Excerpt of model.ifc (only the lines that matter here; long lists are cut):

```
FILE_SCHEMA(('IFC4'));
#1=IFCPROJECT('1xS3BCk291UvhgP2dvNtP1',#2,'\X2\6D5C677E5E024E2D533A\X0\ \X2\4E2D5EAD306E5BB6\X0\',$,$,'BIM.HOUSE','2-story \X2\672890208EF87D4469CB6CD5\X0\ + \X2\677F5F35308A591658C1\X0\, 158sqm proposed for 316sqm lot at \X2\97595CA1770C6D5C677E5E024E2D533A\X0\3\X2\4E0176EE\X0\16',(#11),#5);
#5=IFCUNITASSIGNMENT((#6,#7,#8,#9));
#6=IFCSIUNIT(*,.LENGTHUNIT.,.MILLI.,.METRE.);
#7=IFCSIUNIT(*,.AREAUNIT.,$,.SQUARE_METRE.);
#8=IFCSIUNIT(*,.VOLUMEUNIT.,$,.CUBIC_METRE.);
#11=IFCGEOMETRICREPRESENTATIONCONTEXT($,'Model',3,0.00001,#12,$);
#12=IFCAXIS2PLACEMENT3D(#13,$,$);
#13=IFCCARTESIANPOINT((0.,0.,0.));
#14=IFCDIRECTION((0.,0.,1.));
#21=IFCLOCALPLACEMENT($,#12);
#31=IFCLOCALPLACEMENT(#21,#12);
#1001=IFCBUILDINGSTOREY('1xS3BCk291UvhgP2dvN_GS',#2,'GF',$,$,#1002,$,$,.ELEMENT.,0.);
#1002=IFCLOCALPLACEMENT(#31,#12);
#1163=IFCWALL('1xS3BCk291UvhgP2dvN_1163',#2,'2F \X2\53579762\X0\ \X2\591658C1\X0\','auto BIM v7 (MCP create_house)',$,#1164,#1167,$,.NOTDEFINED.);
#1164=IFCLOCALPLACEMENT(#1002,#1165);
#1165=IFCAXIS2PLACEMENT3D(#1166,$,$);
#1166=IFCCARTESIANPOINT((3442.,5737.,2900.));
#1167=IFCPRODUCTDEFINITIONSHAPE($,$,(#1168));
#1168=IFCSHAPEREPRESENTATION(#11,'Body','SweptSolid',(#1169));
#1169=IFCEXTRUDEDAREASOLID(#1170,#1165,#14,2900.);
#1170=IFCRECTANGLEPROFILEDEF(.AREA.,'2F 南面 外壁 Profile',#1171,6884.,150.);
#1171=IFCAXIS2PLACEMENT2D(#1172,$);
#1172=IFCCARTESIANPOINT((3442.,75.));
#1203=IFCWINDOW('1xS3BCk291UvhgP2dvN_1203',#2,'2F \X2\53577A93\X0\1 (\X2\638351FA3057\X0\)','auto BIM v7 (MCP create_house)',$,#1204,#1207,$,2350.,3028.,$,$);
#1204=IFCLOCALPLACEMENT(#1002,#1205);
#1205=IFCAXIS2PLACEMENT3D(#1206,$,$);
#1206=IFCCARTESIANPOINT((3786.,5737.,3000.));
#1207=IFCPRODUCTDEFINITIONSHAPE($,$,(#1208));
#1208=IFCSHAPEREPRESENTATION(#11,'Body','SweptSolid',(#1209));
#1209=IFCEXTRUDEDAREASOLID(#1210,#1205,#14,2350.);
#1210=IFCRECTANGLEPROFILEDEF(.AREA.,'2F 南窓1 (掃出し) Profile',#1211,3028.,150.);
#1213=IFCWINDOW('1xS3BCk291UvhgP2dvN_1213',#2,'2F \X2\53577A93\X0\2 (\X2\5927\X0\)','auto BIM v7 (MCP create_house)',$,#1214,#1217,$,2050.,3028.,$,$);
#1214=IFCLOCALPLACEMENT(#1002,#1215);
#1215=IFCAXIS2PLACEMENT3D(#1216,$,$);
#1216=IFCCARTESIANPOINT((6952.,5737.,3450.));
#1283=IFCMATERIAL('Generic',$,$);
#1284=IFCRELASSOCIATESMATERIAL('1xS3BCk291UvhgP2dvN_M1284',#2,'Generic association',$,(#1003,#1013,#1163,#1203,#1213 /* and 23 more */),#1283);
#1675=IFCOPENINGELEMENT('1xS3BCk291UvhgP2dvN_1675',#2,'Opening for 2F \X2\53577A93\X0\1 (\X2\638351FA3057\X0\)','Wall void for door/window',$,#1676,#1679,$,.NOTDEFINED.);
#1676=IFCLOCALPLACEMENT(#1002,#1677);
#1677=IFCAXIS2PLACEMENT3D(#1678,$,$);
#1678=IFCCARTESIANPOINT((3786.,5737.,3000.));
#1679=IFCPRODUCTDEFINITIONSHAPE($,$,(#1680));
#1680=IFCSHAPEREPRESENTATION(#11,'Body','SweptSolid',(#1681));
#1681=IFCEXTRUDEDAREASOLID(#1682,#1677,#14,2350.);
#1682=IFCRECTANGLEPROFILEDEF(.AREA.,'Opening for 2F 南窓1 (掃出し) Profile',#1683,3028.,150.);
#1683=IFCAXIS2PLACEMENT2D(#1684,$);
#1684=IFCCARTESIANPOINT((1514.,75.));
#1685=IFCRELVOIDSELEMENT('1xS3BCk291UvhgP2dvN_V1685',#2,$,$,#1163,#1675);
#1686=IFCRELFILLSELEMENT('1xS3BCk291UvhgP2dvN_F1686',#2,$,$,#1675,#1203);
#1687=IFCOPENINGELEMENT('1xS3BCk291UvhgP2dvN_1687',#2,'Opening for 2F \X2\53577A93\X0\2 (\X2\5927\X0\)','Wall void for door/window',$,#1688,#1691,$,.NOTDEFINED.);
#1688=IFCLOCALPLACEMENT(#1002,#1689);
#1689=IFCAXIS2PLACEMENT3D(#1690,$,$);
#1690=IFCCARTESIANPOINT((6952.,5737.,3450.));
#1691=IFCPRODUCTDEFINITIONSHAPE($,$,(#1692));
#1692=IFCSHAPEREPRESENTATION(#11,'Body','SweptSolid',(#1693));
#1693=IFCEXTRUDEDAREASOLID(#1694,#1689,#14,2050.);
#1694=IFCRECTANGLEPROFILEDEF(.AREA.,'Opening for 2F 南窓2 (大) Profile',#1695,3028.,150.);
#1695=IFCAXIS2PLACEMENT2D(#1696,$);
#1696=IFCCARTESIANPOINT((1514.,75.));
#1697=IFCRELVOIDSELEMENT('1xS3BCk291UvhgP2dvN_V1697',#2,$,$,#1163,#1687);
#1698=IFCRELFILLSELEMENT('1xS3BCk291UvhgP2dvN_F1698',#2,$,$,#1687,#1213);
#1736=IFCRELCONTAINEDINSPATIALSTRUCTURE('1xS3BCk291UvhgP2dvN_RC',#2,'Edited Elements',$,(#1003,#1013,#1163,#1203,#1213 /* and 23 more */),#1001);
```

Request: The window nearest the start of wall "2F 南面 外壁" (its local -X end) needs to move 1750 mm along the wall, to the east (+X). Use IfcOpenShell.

```python
import ifcopenshell
import ifcopenshell.api.geometry
import ifcopenshell.util.placement

model = ifcopenshell.open("model.ifc")

window = model.by_id(1203)
opening = window.FillsVoids[0].RelatingOpeningElement
wall = opening.VoidsElements[0].RelatingBuildingElement

wall_matrix = ifcopenshell.util.placement.get_local_placement(wall.ObjectPlacement)
shift = wall_matrix[:3, 0] * 1750.0
before = ifcopenshell.util.placement.get_local_placement(window.ObjectPlacement)[:3, 3].copy()

# The window is not placed relative to its opening, so move both.
for product in (opening, window):
    matrix = ifcopenshell.util.placement.get_local_placement(product.ObjectPlacement)
    matrix[:3, 3] += shift
    ifcopenshell.api.geometry.edit_object_placement(model, product=product, matrix=matrix, is_si=False)

after = ifcopenshell.util.placement.get_local_placement(window.ObjectPlacement)[:3, 3]
print("window moved by", (after - before).round(3) + 0.0)

model.write("model_edited.ifc")
```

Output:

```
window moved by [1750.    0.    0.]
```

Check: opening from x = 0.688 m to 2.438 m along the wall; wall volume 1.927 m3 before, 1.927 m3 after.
